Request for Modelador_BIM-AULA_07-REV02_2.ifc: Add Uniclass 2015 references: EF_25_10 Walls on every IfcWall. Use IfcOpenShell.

First a look at what the model holds.

```python
import ifcopenshell

model = ifcopenshell.open("Modelador_BIM-AULA_07-REV02_2.ifc")
print(model.schema)
print("classifications:", [c.Name for c in model.by_type("IfcClassification")])
for ifc_class in ("IfcDoor", "IfcRoof", "IfcStair", "IfcWall", "IfcWindow"):
    print(ifc_class, len(model.by_type(ifc_class)))
```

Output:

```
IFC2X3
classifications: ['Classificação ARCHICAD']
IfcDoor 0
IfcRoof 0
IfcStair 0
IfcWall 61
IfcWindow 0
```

```python
import ifcopenshell
import ifcopenshell.api.classification

model = ifcopenshell.open("Modelador_BIM-AULA_07-REV02_2.ifc")

# IFC2X3 requires Source and Edition and has no link from the project to the system.
system = model.create_entity("IfcClassification", Source="NBS", Edition="2015", Name="Uniclass 2015")

codes = {
    "IfcWall": ("EF_25_10", "Walls"),
}
for ifc_class, (code, name) in codes.items():
    products = model.by_type(ifc_class)
    ifcopenshell.api.classification.add_reference(
        model, products=products, classification=system, identification=code, name=name
    )
    print(code, len(products))

model.write("Modelador_BIM-AULA_07-REV02_2_edited.ifc")
```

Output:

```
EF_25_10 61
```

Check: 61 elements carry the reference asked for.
